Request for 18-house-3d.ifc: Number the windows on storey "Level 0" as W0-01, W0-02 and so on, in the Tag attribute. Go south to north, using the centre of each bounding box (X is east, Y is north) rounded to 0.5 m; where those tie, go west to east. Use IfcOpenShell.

First a look at what the model holds.

```python
import ifcopenshell
import ifcopenshell.util.element
import ifcopenshell.util.placement

model = ifcopenshell.open("18-house-3d.ifc")
print(model.schema)
storey = next(s for s in model.by_type("IfcBuildingStorey") if s.Name == "Level 0")
windows = [e for e in ifcopenshell.util.element.get_decomposition(storey) if e.is_a("IfcWindow")]
for e in sorted(windows, key=lambda e: e.id()):
    origin = ifcopenshell.util.placement.get_local_placement(e.ObjectPlacement)[:3, 3]
    print(e.id(), e.Tag, e.Name, origin.round(2) + 0.0, sep=" | ")
```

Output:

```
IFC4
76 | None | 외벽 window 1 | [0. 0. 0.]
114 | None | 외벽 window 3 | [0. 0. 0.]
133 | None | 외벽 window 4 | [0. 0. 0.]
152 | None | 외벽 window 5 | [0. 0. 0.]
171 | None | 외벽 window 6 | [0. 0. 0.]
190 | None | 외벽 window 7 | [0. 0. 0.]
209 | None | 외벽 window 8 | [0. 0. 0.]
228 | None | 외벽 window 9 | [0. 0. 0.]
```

```python
import ifcopenshell
import ifcopenshell.geom
import ifcopenshell.util.element
import ifcopenshell.util.shape

model = ifcopenshell.open("18-house-3d.ifc")
settings = ifcopenshell.geom.settings()
settings.set("use-world-coords", True)


def centre(element):
    shape = ifcopenshell.geom.create_shape(settings, element)
    return ifcopenshell.util.shape.get_bbox_centroid(shape.geometry)


storey = next(s for s in model.by_type("IfcBuildingStorey") if s.Name == "Level 0")
windows = [e for e in ifcopenshell.util.element.get_decomposition(storey) if e.is_a("IfcWindow")]

# Insertion points can sit at a corner or the storey origin, so sort by the geometry (in metres).
centres = {e: centre(e) for e in windows}
windows.sort(key=lambda e: (round(centres[e][1] / 0.5), centres[e][0]))

for i, e in enumerate(windows, start=1):
    number = f"W0-{i:02d}"
    e.Tag = number
    print(e.id(), number)

model.write("18-house-3d_edited.ifc")
```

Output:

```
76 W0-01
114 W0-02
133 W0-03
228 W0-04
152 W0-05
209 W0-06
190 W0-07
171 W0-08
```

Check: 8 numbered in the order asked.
